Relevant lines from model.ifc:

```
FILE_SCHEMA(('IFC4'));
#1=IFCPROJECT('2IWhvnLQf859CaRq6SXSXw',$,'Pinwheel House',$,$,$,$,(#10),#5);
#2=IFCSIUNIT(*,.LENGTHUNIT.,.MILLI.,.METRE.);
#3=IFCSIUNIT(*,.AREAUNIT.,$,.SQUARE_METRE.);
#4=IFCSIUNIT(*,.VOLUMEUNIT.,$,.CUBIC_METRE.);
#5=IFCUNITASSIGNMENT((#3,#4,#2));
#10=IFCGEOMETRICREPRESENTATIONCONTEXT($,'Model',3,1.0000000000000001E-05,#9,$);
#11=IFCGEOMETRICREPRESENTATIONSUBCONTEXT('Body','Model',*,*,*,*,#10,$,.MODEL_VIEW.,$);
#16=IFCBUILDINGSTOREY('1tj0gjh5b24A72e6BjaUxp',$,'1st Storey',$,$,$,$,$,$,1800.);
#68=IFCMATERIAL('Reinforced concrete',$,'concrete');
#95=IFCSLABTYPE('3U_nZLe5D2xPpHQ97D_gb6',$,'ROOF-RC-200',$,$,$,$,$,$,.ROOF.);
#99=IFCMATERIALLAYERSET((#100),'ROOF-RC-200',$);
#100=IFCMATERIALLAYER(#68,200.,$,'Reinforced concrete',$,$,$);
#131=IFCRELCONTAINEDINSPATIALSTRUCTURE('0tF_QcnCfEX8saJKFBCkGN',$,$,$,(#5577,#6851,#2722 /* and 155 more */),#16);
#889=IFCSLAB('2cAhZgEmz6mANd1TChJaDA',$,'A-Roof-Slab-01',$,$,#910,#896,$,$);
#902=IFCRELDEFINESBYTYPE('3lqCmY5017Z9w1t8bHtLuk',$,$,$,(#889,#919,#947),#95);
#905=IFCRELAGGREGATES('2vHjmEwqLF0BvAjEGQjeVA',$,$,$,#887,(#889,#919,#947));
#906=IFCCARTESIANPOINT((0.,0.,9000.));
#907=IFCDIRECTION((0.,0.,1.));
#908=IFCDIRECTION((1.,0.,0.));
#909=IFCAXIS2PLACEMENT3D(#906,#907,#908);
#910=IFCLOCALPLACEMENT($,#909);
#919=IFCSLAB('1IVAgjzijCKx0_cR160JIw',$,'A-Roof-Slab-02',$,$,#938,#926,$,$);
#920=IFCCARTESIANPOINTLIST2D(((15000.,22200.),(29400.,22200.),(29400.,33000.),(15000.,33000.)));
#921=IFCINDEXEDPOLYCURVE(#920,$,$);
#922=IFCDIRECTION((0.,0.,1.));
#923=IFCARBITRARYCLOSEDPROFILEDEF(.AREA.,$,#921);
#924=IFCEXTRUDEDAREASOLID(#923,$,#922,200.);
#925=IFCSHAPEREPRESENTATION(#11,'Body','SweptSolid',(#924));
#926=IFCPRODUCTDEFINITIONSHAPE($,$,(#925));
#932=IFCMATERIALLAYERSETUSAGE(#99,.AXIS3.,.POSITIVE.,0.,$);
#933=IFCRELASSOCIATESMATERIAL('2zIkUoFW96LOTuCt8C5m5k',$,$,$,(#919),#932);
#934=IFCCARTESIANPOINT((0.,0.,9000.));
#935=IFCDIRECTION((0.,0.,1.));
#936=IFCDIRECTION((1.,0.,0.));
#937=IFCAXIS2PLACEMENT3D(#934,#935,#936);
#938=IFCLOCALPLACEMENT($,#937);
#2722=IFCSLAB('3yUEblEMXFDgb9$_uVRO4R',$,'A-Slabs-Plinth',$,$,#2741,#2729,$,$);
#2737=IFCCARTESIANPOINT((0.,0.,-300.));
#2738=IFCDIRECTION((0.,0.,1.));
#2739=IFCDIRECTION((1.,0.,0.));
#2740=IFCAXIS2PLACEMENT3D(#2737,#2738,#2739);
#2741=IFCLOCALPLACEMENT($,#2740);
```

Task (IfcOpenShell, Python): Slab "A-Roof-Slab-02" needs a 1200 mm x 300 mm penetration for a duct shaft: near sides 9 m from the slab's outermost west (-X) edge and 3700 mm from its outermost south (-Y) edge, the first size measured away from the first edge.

```python
import numpy as np
import ifcopenshell
import ifcopenshell.api.feature
import ifcopenshell.api.geometry
import ifcopenshell.api.root
import ifcopenshell.geom
import ifcopenshell.util.placement
import ifcopenshell.util.representation
import ifcopenshell.util.shape
import ifcopenshell.util.unit

model = ifcopenshell.open("model.ifc")
unit_scale = ifcopenshell.util.unit.calculate_unit_scale(model)
settings = ifcopenshell.geom.settings()


def volume(element):
    """Net volume in cubic metres, openings subtracted."""
    shape = ifcopenshell.geom.create_shape(settings, element)
    return ifcopenshell.util.shape.get_volume(shape.geometry)


slab = model.by_id(919)
before = volume(slab)

# Extent in the slab's own axes, in metres. The edges named are its -X and -Y sides.
slab_shape = ifcopenshell.geom.create_shape(settings, slab)
vertices = ifcopenshell.util.shape.get_vertices(slab_shape.geometry)
x_min, y_min, bottom = vertices.min(axis=0)
top = vertices[:, 2].max()

opening = ifcopenshell.api.root.create_entity(model, ifc_class="IfcOpeningElement", name="Duct shaft opening", predefined_type="OPENING")
context = ifcopenshell.util.representation.get_context(model, "Model", "Body", "MODEL_VIEW")
width, depth = 1.2, 0.3
outline = [(0.0, 0.0), (width, 0.0), (width, depth), (0.0, depth), (0.0, 0.0)]
# Overshoot both faces by 50 mm so the cut is clean.
shape = ifcopenshell.api.geometry.add_slab_representation(
    model, context=context, depth=top - bottom + 0.1, polyline=outline
)
ifcopenshell.api.geometry.assign_representation(model, product=opening, representation=shape)

matrix = ifcopenshell.util.placement.get_local_placement(slab.ObjectPlacement)
matrix[:, 3] = matrix @ np.append(np.array([x_min + 9, y_min + 3.7, bottom - 0.05]) / unit_scale, 1.0)
ifcopenshell.api.geometry.edit_object_placement(model, product=opening, matrix=matrix, is_si=False)
ifcopenshell.api.feature.add_feature(model, feature=opening, element=slab)

after = volume(slab)

print(f"slab volume {before:.3f} -> {after:.3f} m3")

model.write("model_updated.ifc")
```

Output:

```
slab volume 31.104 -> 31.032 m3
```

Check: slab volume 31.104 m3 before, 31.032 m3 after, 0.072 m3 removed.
